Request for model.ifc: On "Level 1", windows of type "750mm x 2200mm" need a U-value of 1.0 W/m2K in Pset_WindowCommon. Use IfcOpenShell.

First a look at what the model holds.

```python
import ifcopenshell
import ifcopenshell.util.element

model = ifcopenshell.open("model.ifc")
print(model.schema)
storey = next(s for s in model.by_type("IfcBuildingStorey") if s.Name == "Level 1")
windows = [e for e in ifcopenshell.util.element.get_decomposition(storey) if e.is_a("IfcWindow")]
seen = {}
for e in windows:
    element_type = ifcopenshell.util.element.get_type(e)
    key = (element_type.Name if element_type != e and element_type else None, ifcopenshell.util.element.get_pset(e, "Pset_WindowCommon", "ThermalTransmittance"))
    seen[key] = seen.get(key, 0) + 1
for (name, value), count in sorted(seen.items(), key=str):
    print(count, "x", name, "|", value)
```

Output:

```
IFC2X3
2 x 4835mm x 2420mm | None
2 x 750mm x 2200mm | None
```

```python
import ifcopenshell
import ifcopenshell.api.pset
import ifcopenshell.util.element

model = ifcopenshell.open("model.ifc")

storey = next(s for s in model.by_type("IfcBuildingStorey") if s.Name == "Level 1")
windows = [e for e in ifcopenshell.util.element.get_decomposition(storey) if e.is_a("IfcWindow")]

count = 0
for e in windows:
    element_type = ifcopenshell.util.element.get_type(e)
    if element_type in (None, e) or element_type.Name != "750mm x 2200mm":
        continue
    # add_pset returns the element's existing set when there is one.
    pset = ifcopenshell.api.pset.add_pset(model, product=e, name="Pset_WindowCommon")
    ifcopenshell.api.pset.edit_pset(model, pset=pset, properties={"ThermalTransmittance": 1.0})
    count += 1

print(count, "windows updated")

model.write("model_edited.ifc")
```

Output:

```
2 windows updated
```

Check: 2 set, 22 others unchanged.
